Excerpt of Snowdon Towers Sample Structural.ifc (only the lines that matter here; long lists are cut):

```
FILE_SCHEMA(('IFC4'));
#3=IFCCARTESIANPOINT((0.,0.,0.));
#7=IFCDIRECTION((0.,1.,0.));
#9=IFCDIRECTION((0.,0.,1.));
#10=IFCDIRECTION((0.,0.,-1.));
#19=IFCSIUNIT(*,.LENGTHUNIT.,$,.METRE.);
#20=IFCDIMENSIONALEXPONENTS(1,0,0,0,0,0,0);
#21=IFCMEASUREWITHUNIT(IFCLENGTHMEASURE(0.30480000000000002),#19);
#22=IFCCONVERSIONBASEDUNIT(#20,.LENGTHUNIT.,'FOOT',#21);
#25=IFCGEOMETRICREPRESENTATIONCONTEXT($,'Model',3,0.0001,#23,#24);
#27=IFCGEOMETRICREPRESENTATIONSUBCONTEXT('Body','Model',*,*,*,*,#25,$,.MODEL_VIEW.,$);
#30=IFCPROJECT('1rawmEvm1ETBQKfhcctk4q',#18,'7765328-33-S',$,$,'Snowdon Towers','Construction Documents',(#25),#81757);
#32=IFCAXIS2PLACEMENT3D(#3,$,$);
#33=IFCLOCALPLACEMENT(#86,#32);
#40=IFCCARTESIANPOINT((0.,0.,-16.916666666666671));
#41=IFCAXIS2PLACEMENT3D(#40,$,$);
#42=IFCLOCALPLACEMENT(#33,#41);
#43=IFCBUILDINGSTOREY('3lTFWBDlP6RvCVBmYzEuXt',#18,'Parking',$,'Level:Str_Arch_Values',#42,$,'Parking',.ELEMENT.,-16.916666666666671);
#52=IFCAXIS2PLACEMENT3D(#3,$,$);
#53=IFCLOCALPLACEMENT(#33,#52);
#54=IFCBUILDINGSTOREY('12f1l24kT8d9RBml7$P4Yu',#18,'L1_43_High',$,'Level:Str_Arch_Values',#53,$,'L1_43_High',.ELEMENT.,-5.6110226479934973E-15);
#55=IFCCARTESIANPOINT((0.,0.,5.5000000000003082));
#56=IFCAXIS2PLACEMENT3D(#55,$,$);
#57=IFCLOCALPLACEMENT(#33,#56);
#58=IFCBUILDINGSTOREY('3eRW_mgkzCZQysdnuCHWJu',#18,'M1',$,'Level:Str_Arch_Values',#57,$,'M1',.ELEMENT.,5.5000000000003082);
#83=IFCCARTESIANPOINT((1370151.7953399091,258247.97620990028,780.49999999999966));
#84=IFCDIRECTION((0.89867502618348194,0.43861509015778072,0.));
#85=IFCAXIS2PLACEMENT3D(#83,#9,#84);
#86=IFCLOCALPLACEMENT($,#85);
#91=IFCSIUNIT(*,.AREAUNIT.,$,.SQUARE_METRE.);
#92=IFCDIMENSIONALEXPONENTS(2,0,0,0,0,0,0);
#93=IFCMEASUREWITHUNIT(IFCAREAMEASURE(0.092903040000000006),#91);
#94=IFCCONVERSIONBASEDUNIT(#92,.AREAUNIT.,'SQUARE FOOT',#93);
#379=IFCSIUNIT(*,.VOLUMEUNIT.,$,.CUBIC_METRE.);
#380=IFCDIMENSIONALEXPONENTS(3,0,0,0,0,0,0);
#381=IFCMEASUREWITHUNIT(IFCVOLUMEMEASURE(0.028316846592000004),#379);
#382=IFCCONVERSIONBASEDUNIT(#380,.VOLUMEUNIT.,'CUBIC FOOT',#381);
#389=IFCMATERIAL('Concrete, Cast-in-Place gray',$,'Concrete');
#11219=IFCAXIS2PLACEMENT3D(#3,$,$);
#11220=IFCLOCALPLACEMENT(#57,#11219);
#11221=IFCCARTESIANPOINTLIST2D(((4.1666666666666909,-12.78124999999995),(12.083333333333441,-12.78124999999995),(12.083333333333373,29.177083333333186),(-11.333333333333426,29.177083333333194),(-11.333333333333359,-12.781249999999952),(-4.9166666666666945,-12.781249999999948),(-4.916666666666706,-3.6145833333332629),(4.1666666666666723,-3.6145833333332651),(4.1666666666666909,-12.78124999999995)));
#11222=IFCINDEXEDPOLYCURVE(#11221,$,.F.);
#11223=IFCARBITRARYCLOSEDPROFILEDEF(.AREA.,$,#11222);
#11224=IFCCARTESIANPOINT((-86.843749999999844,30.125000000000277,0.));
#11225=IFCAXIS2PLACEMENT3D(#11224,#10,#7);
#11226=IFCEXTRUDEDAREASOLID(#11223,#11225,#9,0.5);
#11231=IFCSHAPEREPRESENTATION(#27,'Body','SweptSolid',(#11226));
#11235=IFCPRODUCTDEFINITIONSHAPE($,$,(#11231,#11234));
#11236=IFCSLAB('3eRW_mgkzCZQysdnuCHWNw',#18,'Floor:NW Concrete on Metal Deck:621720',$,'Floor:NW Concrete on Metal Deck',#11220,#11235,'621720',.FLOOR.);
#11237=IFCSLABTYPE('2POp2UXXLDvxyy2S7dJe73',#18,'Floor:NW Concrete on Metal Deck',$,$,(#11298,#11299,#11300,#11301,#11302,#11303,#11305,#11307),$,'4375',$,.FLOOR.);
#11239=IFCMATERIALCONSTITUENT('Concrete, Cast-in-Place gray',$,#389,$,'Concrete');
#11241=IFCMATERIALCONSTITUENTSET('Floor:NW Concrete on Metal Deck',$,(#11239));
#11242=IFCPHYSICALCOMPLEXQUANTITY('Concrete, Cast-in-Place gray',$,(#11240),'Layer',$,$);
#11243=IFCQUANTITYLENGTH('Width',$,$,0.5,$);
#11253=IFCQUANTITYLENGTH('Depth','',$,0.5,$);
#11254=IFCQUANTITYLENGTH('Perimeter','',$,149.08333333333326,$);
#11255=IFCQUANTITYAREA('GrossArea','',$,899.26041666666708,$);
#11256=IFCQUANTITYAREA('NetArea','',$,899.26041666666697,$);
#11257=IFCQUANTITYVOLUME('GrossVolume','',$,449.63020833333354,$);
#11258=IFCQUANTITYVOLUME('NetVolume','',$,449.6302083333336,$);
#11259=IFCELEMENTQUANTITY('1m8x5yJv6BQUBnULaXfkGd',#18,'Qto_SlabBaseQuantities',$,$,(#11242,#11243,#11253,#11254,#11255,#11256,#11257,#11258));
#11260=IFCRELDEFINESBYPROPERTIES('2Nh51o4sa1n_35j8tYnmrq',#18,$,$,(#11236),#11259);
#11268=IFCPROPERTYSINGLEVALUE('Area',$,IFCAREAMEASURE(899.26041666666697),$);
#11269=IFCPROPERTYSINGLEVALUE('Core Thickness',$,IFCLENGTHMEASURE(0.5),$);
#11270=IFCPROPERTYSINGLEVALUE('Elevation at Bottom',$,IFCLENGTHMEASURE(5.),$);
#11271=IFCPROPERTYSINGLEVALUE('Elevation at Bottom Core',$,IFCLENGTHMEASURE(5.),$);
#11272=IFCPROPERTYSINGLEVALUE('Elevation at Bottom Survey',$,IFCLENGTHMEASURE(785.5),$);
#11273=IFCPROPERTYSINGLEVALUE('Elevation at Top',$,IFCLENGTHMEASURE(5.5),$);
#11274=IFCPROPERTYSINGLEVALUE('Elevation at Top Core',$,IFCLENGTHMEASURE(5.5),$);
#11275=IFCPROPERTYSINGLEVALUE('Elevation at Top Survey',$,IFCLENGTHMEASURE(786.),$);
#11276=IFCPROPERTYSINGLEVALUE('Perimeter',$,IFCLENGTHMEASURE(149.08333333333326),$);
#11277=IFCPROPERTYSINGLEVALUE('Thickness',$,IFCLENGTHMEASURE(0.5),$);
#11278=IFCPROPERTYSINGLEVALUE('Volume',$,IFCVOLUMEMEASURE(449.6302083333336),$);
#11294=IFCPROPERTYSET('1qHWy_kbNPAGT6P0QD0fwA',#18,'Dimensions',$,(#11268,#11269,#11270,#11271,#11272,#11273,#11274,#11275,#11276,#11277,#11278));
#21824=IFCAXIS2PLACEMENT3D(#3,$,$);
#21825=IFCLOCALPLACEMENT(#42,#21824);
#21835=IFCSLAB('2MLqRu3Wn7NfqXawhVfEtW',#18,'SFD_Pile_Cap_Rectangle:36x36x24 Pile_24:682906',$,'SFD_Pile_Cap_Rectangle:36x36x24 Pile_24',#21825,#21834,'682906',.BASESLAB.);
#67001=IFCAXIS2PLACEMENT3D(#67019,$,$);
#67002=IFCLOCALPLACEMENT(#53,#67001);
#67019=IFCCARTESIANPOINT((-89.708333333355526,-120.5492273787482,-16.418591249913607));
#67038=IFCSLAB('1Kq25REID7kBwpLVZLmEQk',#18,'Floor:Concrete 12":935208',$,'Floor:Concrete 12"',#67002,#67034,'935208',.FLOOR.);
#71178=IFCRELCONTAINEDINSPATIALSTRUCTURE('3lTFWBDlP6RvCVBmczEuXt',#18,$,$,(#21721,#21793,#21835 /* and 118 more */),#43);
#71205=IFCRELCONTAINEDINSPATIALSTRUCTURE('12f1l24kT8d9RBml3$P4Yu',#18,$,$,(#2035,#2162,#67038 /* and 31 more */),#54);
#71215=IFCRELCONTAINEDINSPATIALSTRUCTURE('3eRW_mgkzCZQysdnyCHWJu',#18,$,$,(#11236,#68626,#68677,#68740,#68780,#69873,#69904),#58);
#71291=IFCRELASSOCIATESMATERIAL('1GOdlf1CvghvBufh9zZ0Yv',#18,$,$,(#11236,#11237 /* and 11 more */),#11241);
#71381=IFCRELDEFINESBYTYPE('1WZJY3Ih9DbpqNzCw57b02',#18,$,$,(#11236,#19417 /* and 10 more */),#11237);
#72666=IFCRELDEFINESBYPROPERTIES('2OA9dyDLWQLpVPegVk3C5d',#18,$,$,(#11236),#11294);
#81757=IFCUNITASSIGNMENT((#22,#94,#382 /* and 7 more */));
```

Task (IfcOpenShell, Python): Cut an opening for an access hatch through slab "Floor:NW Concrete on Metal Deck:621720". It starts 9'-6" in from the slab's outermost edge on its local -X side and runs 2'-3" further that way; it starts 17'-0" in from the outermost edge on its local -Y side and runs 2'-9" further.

```python
import numpy as np
import ifcopenshell
import ifcopenshell.api.feature
import ifcopenshell.api.geometry
import ifcopenshell.api.pset
import ifcopenshell.api.root
import ifcopenshell.geom
import ifcopenshell.util.element
import ifcopenshell.util.placement
import ifcopenshell.util.representation
import ifcopenshell.util.shape
import ifcopenshell.util.unit

model = ifcopenshell.open("Snowdon Towers Sample Structural.ifc")
unit_scale = ifcopenshell.util.unit.calculate_unit_scale(model)
area_scale = ifcopenshell.util.unit.calculate_unit_scale(model, "AREAUNIT")
volume_scale = ifcopenshell.util.unit.calculate_unit_scale(model, "VOLUMEUNIT")
settings = ifcopenshell.geom.settings()


def volume(element):
    """Net volume in cubic metres, openings subtracted."""
    shape = ifcopenshell.geom.create_shape(settings, element)
    return ifcopenshell.util.shape.get_volume(shape.geometry)


slab = model.by_guid("3eRW_mgkzCZQysdnuCHWNw")
before = volume(slab)

# Extent in the slab's own axes, in metres. The edges named are its -X and -Y sides.
slab_shape = ifcopenshell.geom.create_shape(settings, slab)
vertices = ifcopenshell.util.shape.get_vertices(slab_shape.geometry)
x_min, y_min, bottom = vertices.min(axis=0)
top = vertices[:, 2].max()

opening = ifcopenshell.api.root.create_entity(model, ifc_class="IfcOpeningElement", name="Access hatch opening", predefined_type="OPENING")
context = ifcopenshell.util.representation.get_context(model, "Model", "Body", "MODEL_VIEW")
width, depth = 0.6858, 0.8382
outline = [(0.0, 0.0), (width, 0.0), (width, depth), (0.0, depth), (0.0, 0.0)]
# Overshoot both faces by 50 mm so the cut is clean.
shape = ifcopenshell.api.geometry.add_slab_representation(
    model, context=context, depth=top - bottom + 0.1, polyline=outline
)
ifcopenshell.api.geometry.assign_representation(model, product=opening, representation=shape)

matrix = ifcopenshell.util.placement.get_local_placement(slab.ObjectPlacement)
matrix[:, 3] = matrix @ np.append(np.array([x_min + 2.8956, y_min + 5.1816, bottom - 0.05]) / unit_scale, 1.0)
ifcopenshell.api.geometry.edit_object_placement(model, product=opening, matrix=matrix, is_si=False)
ifcopenshell.api.feature.add_feature(model, feature=opening, element=slab)

after = volume(slab)

# Update the slab's stored quantities.
qto = model.by_id(ifcopenshell.util.element.get_pset(slab, "Qto_SlabBaseQuantities", should_inherit=False)["id"])
ifcopenshell.api.pset.edit_qto(model, qto=qto, properties={
    "NetArea": after / (top - bottom) / area_scale,
    "NetVolume": after / volume_scale,
})
pset = model.by_id(ifcopenshell.util.element.get_pset(slab, "Dimensions", should_inherit=False)["id"])
ifcopenshell.api.pset.edit_pset(model, pset=pset, properties={
    "Area": model.create_entity("IfcAreaMeasure", after / (top - bottom) / area_scale),
    "Volume": model.create_entity("IfcVolumeMeasure", after / volume_scale),
})

print(f"slab volume {before:.3f} -> {after:.3f} m3")

model.write("Snowdon Towers Sample Structural_edited.ifc")
```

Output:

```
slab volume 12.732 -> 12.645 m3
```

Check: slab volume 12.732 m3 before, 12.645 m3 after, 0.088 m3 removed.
